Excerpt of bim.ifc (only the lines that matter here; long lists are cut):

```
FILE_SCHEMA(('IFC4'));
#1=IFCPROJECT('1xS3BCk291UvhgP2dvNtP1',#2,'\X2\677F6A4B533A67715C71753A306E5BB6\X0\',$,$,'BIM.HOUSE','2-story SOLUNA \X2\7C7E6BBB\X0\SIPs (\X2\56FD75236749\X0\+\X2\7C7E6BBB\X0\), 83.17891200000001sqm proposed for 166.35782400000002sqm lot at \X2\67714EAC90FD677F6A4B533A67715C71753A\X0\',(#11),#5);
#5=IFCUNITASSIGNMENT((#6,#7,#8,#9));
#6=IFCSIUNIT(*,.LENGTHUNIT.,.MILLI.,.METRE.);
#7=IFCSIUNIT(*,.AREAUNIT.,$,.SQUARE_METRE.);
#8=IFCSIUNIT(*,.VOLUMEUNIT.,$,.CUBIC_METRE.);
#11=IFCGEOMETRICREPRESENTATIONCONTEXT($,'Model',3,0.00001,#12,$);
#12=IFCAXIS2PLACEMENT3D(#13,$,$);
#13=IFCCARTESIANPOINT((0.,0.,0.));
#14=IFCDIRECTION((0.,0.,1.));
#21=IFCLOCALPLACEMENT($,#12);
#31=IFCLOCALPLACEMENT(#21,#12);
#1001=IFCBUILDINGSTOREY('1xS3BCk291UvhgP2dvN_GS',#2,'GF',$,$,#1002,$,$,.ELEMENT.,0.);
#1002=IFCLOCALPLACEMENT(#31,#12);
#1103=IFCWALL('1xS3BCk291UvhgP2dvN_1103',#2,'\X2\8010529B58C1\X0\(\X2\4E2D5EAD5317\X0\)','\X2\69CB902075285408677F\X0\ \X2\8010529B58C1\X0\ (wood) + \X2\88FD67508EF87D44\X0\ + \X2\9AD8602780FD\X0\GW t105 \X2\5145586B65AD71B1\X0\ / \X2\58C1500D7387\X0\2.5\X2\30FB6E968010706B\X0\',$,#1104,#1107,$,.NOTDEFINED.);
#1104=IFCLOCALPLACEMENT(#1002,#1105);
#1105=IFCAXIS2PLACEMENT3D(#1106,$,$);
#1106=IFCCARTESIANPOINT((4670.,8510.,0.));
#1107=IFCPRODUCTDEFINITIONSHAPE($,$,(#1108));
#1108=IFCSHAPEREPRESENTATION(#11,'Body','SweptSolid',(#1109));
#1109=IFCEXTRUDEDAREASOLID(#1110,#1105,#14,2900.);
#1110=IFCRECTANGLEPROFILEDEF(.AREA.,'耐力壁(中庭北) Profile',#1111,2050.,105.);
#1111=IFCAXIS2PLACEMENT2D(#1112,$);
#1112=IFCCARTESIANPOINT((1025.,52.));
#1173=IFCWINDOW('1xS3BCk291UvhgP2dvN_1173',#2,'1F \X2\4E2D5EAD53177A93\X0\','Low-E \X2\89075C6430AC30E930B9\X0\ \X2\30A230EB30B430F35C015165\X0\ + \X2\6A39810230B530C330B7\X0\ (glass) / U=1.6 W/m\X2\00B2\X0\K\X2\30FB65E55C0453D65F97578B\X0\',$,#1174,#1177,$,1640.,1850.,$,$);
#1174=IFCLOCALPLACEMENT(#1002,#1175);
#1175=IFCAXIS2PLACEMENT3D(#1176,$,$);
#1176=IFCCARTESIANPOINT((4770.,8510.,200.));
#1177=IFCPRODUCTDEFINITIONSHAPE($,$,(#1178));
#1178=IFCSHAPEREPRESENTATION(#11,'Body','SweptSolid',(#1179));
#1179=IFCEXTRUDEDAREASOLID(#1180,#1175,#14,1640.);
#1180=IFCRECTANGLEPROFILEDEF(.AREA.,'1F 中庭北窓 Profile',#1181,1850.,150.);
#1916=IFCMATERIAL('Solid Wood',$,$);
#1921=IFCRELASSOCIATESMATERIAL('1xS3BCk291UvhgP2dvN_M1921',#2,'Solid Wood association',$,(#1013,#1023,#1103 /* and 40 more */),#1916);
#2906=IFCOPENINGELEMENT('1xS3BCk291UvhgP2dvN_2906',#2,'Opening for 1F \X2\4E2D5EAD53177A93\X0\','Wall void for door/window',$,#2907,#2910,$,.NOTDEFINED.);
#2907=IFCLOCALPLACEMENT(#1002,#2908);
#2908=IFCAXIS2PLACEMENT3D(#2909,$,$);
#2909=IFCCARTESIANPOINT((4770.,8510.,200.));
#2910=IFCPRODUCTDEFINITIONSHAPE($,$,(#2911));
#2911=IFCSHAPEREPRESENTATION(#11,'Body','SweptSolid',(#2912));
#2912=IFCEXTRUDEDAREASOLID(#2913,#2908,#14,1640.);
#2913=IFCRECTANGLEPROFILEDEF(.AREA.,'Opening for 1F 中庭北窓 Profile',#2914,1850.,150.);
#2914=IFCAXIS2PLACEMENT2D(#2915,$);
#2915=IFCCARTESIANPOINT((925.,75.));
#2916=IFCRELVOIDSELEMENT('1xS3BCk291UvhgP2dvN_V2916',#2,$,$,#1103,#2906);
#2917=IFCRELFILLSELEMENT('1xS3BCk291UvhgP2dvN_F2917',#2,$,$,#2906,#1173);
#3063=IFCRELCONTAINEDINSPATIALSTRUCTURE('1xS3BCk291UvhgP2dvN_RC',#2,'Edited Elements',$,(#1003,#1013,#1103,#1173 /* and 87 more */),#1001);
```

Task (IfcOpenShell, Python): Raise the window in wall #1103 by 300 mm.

```python
import numpy as np
import ifcopenshell
import ifcopenshell.api.geometry
import ifcopenshell.util.placement
import ifcopenshell.util.unit

model = ifcopenshell.open("bim.ifc")
unit_scale = ifcopenshell.util.unit.calculate_unit_scale(model)

window = model.by_guid("1xS3BCk291UvhgP2dvN_1173")
opening = window.FillsVoids[0].RelatingOpeningElement
dz = 0.3 / unit_scale

shift = np.array([0.0, 0.0, dz])
# The window is not placed relative to its opening, so move both.
for product in (opening, window):
    matrix = ifcopenshell.util.placement.get_local_placement(product.ObjectPlacement)
    matrix[:3, 3] += shift
    ifcopenshell.api.geometry.edit_object_placement(model, product=product, matrix=matrix, is_si=False)

print(f"moved by {dz * unit_scale:+.3f} m")

model.write("bim_updated.ifc")
```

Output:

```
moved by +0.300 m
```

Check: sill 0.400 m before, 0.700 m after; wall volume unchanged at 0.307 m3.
